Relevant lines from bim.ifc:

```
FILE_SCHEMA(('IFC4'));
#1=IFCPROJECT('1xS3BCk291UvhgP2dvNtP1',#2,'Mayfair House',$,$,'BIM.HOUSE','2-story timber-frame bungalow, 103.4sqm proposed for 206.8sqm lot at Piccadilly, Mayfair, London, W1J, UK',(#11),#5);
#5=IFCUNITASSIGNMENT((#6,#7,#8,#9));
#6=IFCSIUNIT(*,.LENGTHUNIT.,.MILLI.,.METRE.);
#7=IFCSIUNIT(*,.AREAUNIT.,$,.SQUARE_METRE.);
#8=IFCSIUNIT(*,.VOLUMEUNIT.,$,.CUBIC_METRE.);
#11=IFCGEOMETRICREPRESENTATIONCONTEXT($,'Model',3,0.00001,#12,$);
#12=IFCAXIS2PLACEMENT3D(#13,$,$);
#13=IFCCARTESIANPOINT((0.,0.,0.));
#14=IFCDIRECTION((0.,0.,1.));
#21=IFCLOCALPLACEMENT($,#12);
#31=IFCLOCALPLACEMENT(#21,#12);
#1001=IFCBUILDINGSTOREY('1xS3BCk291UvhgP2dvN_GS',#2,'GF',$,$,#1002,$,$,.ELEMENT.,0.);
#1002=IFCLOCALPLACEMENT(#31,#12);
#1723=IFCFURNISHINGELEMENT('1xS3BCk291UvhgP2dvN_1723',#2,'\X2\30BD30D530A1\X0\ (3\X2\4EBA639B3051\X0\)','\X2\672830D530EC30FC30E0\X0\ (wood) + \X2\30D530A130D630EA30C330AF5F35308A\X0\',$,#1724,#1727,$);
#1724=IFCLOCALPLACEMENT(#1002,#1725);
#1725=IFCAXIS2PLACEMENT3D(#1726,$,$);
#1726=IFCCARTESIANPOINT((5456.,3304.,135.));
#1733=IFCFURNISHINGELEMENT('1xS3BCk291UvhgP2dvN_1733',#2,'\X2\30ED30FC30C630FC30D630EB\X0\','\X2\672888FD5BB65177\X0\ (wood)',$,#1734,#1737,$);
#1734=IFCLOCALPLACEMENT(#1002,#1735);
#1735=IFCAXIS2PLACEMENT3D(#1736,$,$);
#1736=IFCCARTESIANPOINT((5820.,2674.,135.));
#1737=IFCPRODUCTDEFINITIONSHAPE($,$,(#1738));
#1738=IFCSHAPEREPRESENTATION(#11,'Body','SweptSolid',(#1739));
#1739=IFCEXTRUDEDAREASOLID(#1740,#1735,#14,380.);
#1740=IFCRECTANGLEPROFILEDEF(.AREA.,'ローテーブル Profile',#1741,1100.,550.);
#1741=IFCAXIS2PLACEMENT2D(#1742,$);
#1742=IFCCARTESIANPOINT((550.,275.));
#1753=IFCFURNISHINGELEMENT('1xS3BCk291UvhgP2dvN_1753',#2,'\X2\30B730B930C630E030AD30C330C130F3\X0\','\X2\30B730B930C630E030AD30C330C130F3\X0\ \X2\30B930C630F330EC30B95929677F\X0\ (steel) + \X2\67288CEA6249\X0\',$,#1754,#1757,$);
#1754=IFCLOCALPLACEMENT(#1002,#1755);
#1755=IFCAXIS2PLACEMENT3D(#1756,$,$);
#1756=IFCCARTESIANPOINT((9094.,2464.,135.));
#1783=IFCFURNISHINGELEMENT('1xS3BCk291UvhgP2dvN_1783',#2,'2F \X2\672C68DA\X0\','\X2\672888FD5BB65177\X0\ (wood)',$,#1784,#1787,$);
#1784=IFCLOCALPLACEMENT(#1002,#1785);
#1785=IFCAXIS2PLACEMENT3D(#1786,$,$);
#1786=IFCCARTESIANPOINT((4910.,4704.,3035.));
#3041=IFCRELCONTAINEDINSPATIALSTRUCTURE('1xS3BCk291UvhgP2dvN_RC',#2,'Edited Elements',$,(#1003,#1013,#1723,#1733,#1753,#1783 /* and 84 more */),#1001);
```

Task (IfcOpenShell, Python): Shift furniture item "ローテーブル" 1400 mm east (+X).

```python
import ifcopenshell
import ifcopenshell.api.geometry
import ifcopenshell.util.placement
import ifcopenshell.util.unit

model = ifcopenshell.open("bim.ifc")
unit_scale = ifcopenshell.util.unit.calculate_unit_scale(model)

item = model.by_guid("1xS3BCk291UvhgP2dvN_1733")
matrix = ifcopenshell.util.placement.get_local_placement(item.ObjectPlacement)
matrix[0, 3] += 1.4 / unit_scale
ifcopenshell.api.geometry.edit_object_placement(model, product=item, matrix=matrix, is_si=False)

print(ifcopenshell.util.placement.get_local_placement(item.ObjectPlacement).round(3) + 0.0)

model.write("bim_rev.ifc")
```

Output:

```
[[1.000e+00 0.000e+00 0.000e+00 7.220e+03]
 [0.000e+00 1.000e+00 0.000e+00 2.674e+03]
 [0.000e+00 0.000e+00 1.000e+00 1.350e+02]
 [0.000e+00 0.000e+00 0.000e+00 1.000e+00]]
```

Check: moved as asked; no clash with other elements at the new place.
